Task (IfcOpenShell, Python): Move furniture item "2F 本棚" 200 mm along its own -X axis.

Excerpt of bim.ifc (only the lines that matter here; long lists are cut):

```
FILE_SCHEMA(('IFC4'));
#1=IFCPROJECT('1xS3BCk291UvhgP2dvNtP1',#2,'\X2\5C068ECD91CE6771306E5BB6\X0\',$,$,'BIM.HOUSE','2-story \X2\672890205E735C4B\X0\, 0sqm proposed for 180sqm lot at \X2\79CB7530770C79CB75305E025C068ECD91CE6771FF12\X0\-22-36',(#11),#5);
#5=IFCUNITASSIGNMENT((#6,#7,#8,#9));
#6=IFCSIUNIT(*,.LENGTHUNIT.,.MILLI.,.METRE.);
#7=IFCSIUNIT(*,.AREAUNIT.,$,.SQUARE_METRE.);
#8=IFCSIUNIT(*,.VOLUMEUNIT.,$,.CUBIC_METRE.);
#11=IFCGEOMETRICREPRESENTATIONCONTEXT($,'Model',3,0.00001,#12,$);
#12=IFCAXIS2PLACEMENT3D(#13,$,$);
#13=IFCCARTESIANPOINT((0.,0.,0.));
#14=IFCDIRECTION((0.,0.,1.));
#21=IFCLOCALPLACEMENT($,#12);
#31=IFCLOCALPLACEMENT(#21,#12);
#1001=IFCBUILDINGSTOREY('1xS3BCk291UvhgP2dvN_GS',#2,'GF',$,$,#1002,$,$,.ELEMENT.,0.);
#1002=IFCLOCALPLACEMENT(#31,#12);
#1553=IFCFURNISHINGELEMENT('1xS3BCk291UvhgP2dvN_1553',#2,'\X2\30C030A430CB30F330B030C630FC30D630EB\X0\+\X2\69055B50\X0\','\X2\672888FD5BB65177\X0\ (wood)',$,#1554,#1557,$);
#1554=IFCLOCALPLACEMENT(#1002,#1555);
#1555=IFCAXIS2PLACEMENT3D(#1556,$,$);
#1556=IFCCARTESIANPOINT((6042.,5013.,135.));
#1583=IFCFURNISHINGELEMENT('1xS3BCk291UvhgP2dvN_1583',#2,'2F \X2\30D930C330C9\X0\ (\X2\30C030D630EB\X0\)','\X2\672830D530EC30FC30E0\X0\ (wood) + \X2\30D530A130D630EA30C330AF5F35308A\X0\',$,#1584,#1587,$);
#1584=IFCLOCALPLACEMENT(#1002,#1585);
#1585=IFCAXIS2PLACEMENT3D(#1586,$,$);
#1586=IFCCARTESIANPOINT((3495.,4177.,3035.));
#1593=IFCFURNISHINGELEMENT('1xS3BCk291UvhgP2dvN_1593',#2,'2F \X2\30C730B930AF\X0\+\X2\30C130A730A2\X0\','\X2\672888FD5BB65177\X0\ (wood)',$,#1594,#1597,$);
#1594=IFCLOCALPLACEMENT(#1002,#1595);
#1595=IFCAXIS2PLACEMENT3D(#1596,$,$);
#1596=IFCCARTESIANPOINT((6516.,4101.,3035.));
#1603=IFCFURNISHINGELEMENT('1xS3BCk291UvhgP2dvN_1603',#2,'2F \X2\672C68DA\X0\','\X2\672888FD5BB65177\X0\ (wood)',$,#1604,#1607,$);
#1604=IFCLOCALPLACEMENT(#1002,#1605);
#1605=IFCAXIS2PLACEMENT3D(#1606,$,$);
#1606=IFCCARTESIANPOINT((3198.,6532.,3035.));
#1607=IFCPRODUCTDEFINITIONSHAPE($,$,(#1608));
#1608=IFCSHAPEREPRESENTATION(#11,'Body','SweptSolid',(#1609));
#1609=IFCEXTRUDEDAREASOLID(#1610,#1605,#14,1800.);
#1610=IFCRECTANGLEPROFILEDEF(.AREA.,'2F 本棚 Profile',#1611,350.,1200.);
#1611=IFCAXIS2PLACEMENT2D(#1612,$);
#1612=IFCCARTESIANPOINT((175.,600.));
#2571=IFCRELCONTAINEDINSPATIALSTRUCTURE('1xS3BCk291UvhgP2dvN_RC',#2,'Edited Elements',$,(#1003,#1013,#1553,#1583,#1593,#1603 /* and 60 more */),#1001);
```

```python
import ifcopenshell
import ifcopenshell.api.geometry
import ifcopenshell.util.placement
import ifcopenshell.util.unit

model = ifcopenshell.open("bim.ifc")
unit_scale = ifcopenshell.util.unit.calculate_unit_scale(model)

item = model.by_guid("1xS3BCk291UvhgP2dvN_1603")
matrix = ifcopenshell.util.placement.get_local_placement(item.ObjectPlacement)
matrix[:3, 3] -= matrix[:3, 0] * 0.2 / unit_scale
ifcopenshell.api.geometry.edit_object_placement(model, product=item, matrix=matrix, is_si=False)

print(ifcopenshell.util.placement.get_local_placement(item.ObjectPlacement).round(3) + 0.0)

model.write("bim_rev.ifc")
```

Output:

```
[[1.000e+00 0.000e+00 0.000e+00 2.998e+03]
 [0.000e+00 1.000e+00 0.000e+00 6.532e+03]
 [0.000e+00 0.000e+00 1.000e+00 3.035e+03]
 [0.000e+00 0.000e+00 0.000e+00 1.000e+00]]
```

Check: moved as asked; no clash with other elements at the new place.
